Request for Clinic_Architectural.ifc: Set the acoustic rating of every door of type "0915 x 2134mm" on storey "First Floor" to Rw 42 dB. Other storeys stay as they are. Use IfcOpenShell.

First a look at what the model holds.

```python
import ifcopenshell
import ifcopenshell.util.element

model = ifcopenshell.open("Clinic_Architectural.ifc")
print(model.schema)
storey = next(s for s in model.by_type("IfcBuildingStorey") if s.Name == "First Floor")
doors = [e for e in ifcopenshell.util.element.get_decomposition(storey) if e.is_a("IfcDoor")]
seen = {}
for e in doors:
    element_type = ifcopenshell.util.element.get_type(e)
    key = (element_type.Name if element_type != e and element_type else None, ifcopenshell.util.element.get_pset(e, "Pset_DoorCommon", "AcousticRating"))
    seen[key] = seen.get(key, 0) + 1
for (name, value), count in sorted(seen.items(), key=str):
    print(count, "x", name, "|", value)
```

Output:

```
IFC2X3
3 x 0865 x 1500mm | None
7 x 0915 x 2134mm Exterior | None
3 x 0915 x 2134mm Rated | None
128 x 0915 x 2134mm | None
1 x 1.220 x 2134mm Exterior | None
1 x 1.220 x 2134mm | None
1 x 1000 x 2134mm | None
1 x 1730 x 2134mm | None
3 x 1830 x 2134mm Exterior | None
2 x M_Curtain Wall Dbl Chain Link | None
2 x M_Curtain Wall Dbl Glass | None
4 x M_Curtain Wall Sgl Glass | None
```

```python
import ifcopenshell
import ifcopenshell.api.pset
import ifcopenshell.util.element

model = ifcopenshell.open("Clinic_Architectural.ifc")

storey = next(s for s in model.by_type("IfcBuildingStorey") if s.Name == "First Floor")
doors = [e for e in ifcopenshell.util.element.get_decomposition(storey) if e.is_a("IfcDoor")]

count = 0
for e in doors:
    element_type = ifcopenshell.util.element.get_type(e)
    if element_type in (None, e) or element_type.Name != "0915 x 2134mm":
        continue
    # add_pset returns the element's existing set when there is one.
    pset = ifcopenshell.api.pset.add_pset(model, product=e, name="Pset_DoorCommon")
    ifcopenshell.api.pset.edit_pset(model, pset=pset, properties={"AcousticRating": "Rw 42 dB"})
    count += 1

print(count, "doors updated")

model.write("Clinic_Architectural_rev.ifc")
```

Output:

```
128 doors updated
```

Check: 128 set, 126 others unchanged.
